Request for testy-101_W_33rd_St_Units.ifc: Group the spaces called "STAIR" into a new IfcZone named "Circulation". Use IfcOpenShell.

First a look at what the model holds.

```python
import ifcopenshell

model = ifcopenshell.open("testy-101_W_33rd_St_Units.ifc")
print(model.schema)
seen = {}
for space in model.by_type("IfcSpace"):
    seen[space.LongName] = seen.get(space.LongName, 0) + 1
for name, count in sorted(seen.items(), key=str):
    print(count, "x", name)
print("zones:", [z.Name for z in model.by_type("IfcZone")][:20])
```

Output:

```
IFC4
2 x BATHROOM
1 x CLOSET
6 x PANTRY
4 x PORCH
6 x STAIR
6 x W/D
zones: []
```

```python
import ifcopenshell
import ifcopenshell.api.group
import ifcopenshell.api.root

model = ifcopenshell.open("testy-101_W_33rd_St_Units.ifc")

names = {"STAIR"}
spaces = [s for s in model.by_type("IfcSpace") if s.LongName in names]

zone = ifcopenshell.api.root.create_entity(model, ifc_class="IfcZone", name="Circulation")
ifcopenshell.api.group.assign_group(model, products=spaces, group=zone)
print(len(spaces), "spaces in", zone.Name)

model.write("testy-101_W_33rd_St_Units_updated.ifc")
```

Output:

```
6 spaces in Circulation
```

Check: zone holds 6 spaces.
